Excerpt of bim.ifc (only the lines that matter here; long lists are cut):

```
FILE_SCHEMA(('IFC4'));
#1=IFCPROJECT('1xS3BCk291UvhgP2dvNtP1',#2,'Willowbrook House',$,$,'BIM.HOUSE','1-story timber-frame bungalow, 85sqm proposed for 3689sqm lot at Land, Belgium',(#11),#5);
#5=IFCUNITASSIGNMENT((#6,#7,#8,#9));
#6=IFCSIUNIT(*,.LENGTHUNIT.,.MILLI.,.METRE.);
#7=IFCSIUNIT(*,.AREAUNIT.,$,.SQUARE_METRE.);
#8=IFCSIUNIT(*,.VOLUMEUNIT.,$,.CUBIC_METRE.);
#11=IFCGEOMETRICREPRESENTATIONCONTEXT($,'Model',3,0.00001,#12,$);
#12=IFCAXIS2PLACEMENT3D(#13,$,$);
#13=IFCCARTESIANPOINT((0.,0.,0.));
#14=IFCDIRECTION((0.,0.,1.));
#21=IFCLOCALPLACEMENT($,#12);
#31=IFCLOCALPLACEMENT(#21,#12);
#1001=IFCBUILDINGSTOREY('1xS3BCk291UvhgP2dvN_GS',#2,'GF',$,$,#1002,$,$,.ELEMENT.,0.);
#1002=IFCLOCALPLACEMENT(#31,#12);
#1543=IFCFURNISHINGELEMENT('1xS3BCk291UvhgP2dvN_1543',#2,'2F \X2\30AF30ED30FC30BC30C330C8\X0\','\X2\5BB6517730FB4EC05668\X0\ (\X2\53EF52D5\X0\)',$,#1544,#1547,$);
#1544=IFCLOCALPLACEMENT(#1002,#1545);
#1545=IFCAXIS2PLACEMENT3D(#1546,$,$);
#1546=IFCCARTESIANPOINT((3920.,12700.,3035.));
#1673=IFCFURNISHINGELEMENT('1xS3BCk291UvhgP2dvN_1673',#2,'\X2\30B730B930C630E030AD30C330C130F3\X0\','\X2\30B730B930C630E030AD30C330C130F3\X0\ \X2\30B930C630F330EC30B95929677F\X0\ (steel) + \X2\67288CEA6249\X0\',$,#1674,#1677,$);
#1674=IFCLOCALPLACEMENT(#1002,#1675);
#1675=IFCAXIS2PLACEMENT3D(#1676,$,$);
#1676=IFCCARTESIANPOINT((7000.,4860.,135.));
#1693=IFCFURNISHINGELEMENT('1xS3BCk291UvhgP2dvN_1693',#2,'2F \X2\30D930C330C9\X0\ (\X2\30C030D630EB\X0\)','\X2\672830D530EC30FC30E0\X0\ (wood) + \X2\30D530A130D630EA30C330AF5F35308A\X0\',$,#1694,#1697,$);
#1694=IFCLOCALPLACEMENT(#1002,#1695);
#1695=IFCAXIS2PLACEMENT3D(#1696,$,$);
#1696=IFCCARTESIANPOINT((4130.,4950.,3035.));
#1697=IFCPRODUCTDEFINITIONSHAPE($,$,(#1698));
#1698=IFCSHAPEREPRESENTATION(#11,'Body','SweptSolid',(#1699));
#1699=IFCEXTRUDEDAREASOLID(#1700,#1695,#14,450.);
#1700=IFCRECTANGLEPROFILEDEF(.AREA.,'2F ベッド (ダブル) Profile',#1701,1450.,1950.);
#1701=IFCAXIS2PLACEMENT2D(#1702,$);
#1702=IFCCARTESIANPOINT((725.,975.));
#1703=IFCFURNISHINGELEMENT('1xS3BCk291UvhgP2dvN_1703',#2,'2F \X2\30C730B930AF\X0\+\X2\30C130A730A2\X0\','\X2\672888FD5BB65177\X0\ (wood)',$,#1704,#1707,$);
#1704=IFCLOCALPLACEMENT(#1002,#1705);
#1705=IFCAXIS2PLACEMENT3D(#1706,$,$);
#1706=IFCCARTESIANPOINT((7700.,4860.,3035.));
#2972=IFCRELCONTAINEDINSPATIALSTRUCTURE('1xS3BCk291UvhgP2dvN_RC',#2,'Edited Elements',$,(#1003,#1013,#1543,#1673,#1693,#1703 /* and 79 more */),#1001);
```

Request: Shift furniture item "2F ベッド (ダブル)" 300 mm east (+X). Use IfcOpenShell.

```python
import ifcopenshell
import ifcopenshell.api.geometry
import ifcopenshell.util.placement
import ifcopenshell.util.unit

model = ifcopenshell.open("bim.ifc")
unit_scale = ifcopenshell.util.unit.calculate_unit_scale(model)

item = model.by_guid("1xS3BCk291UvhgP2dvN_1693")
matrix = ifcopenshell.util.placement.get_local_placement(item.ObjectPlacement)
matrix[0, 3] += 0.3 / unit_scale
ifcopenshell.api.geometry.edit_object_placement(model, product=item, matrix=matrix, is_si=False)

print(ifcopenshell.util.placement.get_local_placement(item.ObjectPlacement).round(3) + 0.0)

model.write("bim_v2.ifc")
```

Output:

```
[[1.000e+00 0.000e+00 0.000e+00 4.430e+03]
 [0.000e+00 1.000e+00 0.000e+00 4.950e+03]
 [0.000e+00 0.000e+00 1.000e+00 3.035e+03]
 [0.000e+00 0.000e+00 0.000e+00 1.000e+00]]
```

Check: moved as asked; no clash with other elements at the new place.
